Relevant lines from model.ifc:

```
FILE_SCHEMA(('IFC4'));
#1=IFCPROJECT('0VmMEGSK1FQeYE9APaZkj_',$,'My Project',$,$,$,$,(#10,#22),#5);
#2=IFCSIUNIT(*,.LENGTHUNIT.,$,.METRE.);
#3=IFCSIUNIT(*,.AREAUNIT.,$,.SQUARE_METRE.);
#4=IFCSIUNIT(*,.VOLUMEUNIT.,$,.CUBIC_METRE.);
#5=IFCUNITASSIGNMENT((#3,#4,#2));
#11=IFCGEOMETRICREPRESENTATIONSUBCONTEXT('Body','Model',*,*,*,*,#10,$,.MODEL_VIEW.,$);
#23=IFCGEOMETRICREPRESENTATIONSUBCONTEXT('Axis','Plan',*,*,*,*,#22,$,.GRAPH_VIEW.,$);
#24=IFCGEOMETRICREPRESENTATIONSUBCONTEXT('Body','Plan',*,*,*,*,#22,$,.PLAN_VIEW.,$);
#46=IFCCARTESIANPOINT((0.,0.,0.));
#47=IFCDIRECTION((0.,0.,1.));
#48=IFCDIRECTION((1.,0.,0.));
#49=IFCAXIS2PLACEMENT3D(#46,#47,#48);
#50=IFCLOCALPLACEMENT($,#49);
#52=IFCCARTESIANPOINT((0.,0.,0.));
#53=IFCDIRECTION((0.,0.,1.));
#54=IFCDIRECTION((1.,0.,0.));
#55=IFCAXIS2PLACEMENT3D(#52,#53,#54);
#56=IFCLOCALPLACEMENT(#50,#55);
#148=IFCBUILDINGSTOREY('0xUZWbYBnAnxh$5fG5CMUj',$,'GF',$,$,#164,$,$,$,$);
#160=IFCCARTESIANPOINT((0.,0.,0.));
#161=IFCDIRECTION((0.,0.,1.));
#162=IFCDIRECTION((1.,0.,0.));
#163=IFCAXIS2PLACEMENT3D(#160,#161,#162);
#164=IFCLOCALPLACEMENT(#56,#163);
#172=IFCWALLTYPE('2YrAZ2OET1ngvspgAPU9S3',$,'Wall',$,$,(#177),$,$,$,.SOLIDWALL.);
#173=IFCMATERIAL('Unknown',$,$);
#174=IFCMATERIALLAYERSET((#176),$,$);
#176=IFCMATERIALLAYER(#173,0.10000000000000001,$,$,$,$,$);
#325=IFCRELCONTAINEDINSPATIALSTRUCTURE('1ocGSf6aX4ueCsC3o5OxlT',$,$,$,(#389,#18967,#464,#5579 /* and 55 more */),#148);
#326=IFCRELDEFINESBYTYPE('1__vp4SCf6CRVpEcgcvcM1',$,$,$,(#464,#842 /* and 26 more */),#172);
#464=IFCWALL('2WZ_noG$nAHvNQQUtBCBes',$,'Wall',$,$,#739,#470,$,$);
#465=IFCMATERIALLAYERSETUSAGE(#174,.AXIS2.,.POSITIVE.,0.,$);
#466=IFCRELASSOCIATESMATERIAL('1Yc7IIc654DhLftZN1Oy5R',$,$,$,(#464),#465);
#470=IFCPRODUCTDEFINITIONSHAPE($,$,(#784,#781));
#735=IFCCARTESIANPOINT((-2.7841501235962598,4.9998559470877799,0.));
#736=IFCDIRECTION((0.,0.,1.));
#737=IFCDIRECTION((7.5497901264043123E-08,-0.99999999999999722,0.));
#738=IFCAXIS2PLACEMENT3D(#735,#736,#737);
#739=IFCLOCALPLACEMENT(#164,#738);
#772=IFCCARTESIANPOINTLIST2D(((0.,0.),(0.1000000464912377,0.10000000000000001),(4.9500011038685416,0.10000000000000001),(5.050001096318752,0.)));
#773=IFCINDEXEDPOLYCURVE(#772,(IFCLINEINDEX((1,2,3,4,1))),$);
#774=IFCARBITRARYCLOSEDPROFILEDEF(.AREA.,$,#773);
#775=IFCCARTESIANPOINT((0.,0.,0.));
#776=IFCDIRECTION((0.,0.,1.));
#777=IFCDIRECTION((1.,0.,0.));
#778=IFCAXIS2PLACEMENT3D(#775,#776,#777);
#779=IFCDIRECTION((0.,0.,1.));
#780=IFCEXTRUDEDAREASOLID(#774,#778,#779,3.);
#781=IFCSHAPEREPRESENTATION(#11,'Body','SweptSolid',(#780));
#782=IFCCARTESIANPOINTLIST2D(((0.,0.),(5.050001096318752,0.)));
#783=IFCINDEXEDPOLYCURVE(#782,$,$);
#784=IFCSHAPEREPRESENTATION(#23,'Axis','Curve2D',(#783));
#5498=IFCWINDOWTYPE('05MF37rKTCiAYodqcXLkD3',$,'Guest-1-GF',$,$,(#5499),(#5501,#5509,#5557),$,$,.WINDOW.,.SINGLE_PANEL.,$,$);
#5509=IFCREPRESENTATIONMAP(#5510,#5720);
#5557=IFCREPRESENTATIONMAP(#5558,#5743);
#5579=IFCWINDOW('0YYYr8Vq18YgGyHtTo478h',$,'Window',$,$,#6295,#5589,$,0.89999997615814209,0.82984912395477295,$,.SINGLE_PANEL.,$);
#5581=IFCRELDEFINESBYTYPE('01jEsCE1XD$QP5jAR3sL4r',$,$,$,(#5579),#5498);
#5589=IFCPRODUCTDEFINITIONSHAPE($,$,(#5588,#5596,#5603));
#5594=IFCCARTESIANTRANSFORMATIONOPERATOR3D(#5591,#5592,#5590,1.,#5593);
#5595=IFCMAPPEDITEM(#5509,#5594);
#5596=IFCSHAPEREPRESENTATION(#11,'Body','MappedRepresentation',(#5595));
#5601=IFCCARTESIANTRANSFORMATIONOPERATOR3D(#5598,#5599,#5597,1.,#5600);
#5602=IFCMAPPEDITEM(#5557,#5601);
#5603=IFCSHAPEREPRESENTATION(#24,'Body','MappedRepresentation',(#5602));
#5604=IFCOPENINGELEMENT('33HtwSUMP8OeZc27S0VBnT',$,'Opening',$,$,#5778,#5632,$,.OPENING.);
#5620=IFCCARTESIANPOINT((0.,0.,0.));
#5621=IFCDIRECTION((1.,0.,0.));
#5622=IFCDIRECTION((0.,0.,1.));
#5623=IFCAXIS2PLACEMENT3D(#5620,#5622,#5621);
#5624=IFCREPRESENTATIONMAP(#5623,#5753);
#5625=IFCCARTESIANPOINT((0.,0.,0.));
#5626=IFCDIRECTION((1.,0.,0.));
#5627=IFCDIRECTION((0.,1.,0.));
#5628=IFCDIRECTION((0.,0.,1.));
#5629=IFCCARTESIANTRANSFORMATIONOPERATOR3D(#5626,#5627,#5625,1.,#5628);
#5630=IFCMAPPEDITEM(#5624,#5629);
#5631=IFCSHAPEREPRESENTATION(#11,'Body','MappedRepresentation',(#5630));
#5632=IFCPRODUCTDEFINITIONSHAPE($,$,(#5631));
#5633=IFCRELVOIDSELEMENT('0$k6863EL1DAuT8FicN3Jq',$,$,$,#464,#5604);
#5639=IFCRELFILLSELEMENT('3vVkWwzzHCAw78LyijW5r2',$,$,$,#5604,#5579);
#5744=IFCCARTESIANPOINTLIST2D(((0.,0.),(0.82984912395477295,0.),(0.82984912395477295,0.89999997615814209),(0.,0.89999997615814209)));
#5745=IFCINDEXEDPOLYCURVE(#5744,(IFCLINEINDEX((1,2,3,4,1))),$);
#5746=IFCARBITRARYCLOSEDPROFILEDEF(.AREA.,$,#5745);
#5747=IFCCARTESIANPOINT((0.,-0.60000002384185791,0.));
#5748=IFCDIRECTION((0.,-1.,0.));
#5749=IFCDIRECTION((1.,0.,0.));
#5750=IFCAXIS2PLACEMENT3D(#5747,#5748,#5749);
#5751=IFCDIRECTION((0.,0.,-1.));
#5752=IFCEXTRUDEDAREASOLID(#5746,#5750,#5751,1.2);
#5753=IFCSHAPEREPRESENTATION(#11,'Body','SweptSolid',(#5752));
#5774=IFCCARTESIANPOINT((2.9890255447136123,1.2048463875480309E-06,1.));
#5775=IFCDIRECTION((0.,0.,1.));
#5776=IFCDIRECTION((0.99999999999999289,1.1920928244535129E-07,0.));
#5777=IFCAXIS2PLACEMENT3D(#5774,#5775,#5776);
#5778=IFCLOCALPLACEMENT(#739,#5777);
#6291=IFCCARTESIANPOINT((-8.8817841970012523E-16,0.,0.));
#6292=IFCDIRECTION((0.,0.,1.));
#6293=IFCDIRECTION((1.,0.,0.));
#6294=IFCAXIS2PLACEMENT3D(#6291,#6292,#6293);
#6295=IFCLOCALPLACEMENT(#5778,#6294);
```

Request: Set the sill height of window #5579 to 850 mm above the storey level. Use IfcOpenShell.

```python
import numpy as np
import ifcopenshell
import ifcopenshell.api.geometry
import ifcopenshell.geom
import ifcopenshell.util.element
import ifcopenshell.util.placement
import ifcopenshell.util.shape
import ifcopenshell.util.unit

model = ifcopenshell.open("model.ifc")
unit_scale = ifcopenshell.util.unit.calculate_unit_scale(model)

window = model.by_guid("0YYYr8Vq18YgGyHtTo478h")
opening = window.FillsVoids[0].RelatingOpeningElement
storey = ifcopenshell.util.element.get_container(window, ifc_class="IfcBuildingStorey")
level = ifcopenshell.util.placement.get_local_placement(storey.ObjectPlacement)[2, 3]

# The opening's origin need not be at the sill, so measure its lowest point.
shape = ifcopenshell.geom.create_shape(ifcopenshell.geom.settings(), opening)
bottom = ifcopenshell.util.shape.get_shape_bottom_elevation(shape, shape.geometry) / unit_scale
dz = level + 0.85 / unit_scale - bottom

shift = np.array([0.0, 0.0, dz])
# The window is placed relative to its opening, so it follows when the opening moves.
matrix = ifcopenshell.util.placement.get_local_placement(opening.ObjectPlacement)
matrix[:3, 3] += shift
ifcopenshell.api.geometry.edit_object_placement(
    model, product=opening, matrix=matrix, is_si=False, should_transform_children=True
)

print(f"moved by {dz * unit_scale:+.3f} m")

model.write("model_v2.ifc")
```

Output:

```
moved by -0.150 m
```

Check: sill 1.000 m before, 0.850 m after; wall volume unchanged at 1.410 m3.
